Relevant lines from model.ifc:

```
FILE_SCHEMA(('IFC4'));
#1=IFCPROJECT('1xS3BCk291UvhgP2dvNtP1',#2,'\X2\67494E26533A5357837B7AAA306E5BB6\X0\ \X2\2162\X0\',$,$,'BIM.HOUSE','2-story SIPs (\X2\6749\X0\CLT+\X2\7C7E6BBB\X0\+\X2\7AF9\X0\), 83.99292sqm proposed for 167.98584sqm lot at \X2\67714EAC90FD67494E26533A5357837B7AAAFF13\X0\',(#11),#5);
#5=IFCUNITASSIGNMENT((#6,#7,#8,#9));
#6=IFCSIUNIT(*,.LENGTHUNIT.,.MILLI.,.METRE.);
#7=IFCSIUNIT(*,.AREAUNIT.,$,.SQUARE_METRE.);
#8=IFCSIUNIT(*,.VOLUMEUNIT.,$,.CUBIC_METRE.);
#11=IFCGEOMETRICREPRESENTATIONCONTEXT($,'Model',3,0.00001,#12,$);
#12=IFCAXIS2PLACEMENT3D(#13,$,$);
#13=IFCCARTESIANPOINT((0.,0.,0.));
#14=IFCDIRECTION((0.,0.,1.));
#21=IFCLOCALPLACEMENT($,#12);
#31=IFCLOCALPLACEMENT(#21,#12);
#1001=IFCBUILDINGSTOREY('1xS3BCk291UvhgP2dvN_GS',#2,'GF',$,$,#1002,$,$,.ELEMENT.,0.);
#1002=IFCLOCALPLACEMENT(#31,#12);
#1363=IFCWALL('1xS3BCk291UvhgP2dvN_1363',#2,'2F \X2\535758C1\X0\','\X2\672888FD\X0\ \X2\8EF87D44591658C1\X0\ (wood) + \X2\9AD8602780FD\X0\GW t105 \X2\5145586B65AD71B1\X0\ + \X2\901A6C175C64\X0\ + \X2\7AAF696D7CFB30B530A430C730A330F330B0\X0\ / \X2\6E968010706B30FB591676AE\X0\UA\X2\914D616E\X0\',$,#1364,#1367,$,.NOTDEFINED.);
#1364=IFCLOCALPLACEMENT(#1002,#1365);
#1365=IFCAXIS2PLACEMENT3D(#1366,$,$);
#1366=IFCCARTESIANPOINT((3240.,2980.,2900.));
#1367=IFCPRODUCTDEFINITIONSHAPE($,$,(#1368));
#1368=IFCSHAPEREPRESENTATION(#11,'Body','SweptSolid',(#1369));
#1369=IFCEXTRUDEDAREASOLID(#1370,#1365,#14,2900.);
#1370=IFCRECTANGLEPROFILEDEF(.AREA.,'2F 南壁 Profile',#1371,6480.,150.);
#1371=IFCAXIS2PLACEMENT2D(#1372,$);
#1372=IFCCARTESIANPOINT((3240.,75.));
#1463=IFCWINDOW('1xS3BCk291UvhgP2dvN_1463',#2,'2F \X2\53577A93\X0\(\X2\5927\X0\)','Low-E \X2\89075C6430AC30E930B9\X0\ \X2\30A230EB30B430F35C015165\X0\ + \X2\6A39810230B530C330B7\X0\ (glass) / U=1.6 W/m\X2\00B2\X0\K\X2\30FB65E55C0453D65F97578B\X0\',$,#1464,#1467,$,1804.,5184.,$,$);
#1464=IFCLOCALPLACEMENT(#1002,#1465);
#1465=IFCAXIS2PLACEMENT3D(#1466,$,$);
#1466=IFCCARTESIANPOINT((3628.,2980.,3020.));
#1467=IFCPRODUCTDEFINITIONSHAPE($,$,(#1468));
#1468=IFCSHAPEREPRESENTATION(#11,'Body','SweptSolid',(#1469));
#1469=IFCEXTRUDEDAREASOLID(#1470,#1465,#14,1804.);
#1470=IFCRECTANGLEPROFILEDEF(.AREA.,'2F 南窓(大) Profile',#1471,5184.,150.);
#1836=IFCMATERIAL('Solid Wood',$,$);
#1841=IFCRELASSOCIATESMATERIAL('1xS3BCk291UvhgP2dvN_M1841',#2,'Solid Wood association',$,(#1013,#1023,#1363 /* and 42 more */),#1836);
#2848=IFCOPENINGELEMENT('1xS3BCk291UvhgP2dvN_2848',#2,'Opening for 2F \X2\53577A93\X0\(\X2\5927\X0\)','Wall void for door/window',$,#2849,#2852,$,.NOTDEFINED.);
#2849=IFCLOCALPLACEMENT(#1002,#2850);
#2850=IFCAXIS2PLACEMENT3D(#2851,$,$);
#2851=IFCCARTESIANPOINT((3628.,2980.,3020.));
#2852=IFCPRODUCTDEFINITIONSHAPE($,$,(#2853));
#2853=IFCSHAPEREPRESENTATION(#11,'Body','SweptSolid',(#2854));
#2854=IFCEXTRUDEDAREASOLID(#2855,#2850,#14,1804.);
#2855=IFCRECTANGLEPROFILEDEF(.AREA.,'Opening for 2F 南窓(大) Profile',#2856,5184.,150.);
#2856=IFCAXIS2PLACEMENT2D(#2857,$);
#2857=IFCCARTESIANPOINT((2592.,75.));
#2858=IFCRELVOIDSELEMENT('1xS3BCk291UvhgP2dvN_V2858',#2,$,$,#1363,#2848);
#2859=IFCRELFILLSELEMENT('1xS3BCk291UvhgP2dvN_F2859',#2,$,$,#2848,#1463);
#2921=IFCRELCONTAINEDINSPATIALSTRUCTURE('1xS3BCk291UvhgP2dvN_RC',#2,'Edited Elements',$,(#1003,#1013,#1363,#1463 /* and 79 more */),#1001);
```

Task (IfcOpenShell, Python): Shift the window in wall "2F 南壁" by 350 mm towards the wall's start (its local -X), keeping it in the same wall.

```python
import ifcopenshell
import ifcopenshell.api.geometry
import ifcopenshell.util.placement
import ifcopenshell.util.unit

model = ifcopenshell.open("model.ifc")
unit_scale = ifcopenshell.util.unit.calculate_unit_scale(model)

window = model.by_guid("1xS3BCk291UvhgP2dvN_1463")
opening = window.FillsVoids[0].RelatingOpeningElement
wall = opening.VoidsElements[0].RelatingBuildingElement

wall_matrix = ifcopenshell.util.placement.get_local_placement(wall.ObjectPlacement)
shift = wall_matrix[:3, 0] * -0.35 / unit_scale
before = ifcopenshell.util.placement.get_local_placement(window.ObjectPlacement)[:3, 3].copy()

# The window is not placed relative to its opening, so move both.
for product in (opening, window):
    matrix = ifcopenshell.util.placement.get_local_placement(product.ObjectPlacement)
    matrix[:3, 3] += shift
    ifcopenshell.api.geometry.edit_object_placement(model, product=product, matrix=matrix, is_si=False)

after = ifcopenshell.util.placement.get_local_placement(window.ObjectPlacement)[:3, 3]
print("window moved by", (after - before).round(3) + 0.0)

model.write("model_updated.ifc")
```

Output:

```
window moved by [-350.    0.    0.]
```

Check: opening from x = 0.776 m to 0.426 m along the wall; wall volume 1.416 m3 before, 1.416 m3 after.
